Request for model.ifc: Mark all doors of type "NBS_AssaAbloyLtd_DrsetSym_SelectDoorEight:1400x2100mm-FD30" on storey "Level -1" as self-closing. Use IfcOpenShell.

First a look at what the model holds.

```python
import ifcopenshell
import ifcopenshell.util.element

model = ifcopenshell.open("model.ifc")
print(model.schema)
storey = next(s for s in model.by_type("IfcBuildingStorey") if s.Name == "Level -1")
doors = [e for e in ifcopenshell.util.element.get_decomposition(storey) if e.is_a("IfcDoor")]
seen = {}
for e in doors:
    element_type = ifcopenshell.util.element.get_type(e)
    key = (element_type.Name if element_type != e and element_type else None, ifcopenshell.util.element.get_pset(e, "Pset_DoorCommon", "SelfClosing"))
    seen[key] = seen.get(key, 0) + 1
for (name, value), count in sorted(seen.items(), key=str):
    print(count, "x", name, "|", value)
```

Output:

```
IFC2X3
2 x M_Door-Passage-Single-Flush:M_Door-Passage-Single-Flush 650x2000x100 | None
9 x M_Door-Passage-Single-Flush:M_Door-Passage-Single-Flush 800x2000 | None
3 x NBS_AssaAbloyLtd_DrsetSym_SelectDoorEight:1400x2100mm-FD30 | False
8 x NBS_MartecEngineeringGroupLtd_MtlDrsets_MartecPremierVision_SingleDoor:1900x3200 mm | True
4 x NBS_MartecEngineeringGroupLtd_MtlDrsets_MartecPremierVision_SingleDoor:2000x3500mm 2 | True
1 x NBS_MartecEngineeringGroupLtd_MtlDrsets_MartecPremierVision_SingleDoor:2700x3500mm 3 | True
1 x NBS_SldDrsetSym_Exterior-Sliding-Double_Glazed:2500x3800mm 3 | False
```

```python
import ifcopenshell
import ifcopenshell.api.pset
import ifcopenshell.util.element

model = ifcopenshell.open("model.ifc")

storey = next(s for s in model.by_type("IfcBuildingStorey") if s.Name == "Level -1")
doors = [e for e in ifcopenshell.util.element.get_decomposition(storey) if e.is_a("IfcDoor")]

count = 0
for e in doors:
    element_type = ifcopenshell.util.element.get_type(e)
    if element_type in (None, e) or element_type.Name != "NBS_AssaAbloyLtd_DrsetSym_SelectDoorEight:1400x2100mm-FD30":
        continue
    # add_pset returns the element's existing set when there is one.
    pset = ifcopenshell.api.pset.add_pset(model, product=e, name="Pset_DoorCommon")
    ifcopenshell.api.pset.edit_pset(model, pset=pset, properties={"SelfClosing": True})
    count += 1

print(count, "doors updated")

model.write("model-out.ifc")
```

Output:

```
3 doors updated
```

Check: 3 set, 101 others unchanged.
